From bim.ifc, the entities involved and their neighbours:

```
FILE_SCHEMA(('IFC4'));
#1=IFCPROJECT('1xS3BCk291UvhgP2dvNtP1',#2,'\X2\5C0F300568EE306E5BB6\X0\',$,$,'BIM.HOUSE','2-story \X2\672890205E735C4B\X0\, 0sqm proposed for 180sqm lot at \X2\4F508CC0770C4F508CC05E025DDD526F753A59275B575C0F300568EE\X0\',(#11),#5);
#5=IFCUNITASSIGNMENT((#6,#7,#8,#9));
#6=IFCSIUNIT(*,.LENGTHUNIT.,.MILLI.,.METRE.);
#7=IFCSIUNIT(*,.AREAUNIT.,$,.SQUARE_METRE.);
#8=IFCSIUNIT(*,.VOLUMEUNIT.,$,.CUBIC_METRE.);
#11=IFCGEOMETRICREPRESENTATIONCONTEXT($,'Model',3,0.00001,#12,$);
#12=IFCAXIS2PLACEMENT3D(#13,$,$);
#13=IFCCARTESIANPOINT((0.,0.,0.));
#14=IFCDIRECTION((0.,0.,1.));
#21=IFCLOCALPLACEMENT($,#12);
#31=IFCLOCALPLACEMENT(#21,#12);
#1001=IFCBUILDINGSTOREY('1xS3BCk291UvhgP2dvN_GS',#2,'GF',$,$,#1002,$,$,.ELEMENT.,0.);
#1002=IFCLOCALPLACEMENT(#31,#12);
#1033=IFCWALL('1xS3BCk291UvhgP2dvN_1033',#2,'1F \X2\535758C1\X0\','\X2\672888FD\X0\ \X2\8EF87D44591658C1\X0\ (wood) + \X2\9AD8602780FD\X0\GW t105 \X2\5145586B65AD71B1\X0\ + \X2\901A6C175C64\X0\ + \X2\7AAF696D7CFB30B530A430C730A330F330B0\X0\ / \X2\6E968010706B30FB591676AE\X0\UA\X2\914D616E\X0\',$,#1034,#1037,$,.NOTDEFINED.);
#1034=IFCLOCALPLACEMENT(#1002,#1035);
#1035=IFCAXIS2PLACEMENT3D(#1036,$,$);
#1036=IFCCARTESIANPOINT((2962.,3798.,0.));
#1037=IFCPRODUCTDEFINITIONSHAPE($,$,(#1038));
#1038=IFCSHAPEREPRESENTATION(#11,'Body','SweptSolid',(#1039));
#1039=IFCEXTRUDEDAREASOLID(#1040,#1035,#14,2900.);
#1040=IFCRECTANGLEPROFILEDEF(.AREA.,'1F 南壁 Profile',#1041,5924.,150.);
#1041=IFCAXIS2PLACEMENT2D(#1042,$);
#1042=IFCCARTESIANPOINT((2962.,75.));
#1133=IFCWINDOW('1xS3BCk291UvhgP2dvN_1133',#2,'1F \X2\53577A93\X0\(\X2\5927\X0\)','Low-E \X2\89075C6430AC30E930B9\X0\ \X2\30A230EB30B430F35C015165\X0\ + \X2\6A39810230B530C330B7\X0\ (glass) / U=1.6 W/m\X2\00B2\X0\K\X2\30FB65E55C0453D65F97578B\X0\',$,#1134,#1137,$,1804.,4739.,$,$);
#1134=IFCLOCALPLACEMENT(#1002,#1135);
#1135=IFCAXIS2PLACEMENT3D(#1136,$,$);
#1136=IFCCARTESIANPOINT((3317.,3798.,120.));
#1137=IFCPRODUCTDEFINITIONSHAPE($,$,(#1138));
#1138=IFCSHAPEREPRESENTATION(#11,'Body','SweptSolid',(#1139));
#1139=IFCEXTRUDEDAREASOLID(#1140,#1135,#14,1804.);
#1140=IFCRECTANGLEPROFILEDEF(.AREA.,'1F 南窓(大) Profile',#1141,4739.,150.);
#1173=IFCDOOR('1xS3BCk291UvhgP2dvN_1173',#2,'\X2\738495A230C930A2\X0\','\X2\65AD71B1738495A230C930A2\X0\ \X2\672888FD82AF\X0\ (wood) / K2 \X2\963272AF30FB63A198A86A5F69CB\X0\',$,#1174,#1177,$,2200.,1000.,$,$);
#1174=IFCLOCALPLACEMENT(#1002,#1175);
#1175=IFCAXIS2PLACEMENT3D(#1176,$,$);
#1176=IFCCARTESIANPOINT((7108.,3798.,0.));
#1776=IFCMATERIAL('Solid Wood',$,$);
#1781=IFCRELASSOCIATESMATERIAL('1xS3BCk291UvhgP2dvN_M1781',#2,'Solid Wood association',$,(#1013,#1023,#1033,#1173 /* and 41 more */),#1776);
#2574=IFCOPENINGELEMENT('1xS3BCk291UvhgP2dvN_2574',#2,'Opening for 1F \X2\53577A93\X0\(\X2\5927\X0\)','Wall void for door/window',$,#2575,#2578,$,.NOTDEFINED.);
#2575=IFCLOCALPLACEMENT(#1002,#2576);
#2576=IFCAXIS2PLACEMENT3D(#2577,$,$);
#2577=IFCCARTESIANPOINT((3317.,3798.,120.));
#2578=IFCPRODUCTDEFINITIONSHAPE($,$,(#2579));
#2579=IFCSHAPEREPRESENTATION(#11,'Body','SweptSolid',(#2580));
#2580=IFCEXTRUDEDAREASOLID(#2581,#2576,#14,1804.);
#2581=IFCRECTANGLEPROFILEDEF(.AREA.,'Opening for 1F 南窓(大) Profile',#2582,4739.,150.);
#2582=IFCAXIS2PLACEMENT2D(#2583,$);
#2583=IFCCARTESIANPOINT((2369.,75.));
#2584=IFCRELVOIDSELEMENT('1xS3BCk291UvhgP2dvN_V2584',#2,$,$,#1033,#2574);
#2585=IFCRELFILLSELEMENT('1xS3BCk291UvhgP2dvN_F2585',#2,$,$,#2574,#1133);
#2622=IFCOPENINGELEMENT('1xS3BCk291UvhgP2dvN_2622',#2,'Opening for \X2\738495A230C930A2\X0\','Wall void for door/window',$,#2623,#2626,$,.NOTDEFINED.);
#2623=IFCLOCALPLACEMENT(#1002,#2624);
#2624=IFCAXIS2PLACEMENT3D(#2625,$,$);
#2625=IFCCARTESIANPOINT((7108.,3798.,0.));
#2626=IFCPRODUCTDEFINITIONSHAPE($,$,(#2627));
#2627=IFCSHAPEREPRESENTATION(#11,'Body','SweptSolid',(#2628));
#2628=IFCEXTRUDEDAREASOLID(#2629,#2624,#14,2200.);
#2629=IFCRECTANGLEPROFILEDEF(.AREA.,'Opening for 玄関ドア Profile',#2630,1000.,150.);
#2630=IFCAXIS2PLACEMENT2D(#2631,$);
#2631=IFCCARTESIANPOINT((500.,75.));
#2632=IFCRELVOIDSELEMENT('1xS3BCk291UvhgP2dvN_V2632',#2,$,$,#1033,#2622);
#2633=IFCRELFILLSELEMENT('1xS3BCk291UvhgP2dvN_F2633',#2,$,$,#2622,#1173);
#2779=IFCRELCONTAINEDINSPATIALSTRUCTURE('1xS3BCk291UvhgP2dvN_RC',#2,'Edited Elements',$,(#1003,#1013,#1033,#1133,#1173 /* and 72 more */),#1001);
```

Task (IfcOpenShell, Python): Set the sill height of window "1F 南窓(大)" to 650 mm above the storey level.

```python
import numpy as np
import ifcopenshell
import ifcopenshell.api.geometry
import ifcopenshell.geom
import ifcopenshell.util.element
import ifcopenshell.util.placement
import ifcopenshell.util.shape
import ifcopenshell.util.unit

model = ifcopenshell.open("bim.ifc")
unit_scale = ifcopenshell.util.unit.calculate_unit_scale(model)

window = model.by_guid("1xS3BCk291UvhgP2dvN_1133")
opening = window.FillsVoids[0].RelatingOpeningElement
storey = ifcopenshell.util.element.get_container(window, ifc_class="IfcBuildingStorey")
level = ifcopenshell.util.placement.get_local_placement(storey.ObjectPlacement)[2, 3]

# The opening's origin need not be at the sill, so measure its lowest point.
shape = ifcopenshell.geom.create_shape(ifcopenshell.geom.settings(), opening)
bottom = ifcopenshell.util.shape.get_shape_bottom_elevation(shape, shape.geometry) / unit_scale
dz = level + 650.0 - bottom

shift = np.array([0.0, 0.0, dz])
# The window is not placed relative to its opening, so move both.
for product in (opening, window):
    matrix = ifcopenshell.util.placement.get_local_placement(product.ObjectPlacement)
    matrix[:3, 3] += shift
    ifcopenshell.api.geometry.edit_object_placement(model, product=product, matrix=matrix, is_si=False)

print(f"moved by {dz * unit_scale:+.3f} m")

model.write("bim_edited.ifc")
```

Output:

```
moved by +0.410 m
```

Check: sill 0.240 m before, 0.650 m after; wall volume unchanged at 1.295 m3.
